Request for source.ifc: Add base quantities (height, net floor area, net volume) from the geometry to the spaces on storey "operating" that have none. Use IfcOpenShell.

First a look at what the model holds.

```python
import ifcopenshell
import ifcopenshell.util.element
import ifcopenshell.util.unit

model = ifcopenshell.open("source.ifc")
print(model.schema)
for unit_type in ("LENGTHUNIT", "AREAUNIT", "VOLUMEUNIT"):
    print(unit_type, ifcopenshell.util.unit.calculate_unit_scale(model, unit_type))
storey = next(s for s in model.by_type("IfcBuildingStorey") if s.Name == "operating")
spaces = [e for e in ifcopenshell.util.element.get_decomposition(storey) if e.is_a("IfcSpace")]
for e in sorted(spaces, key=lambda e: e.id()):
    print(e.id(), e.is_a(), e.Name, list(ifcopenshell.util.element.get_psets(e, qtos_only=True)), sep=" | ")
```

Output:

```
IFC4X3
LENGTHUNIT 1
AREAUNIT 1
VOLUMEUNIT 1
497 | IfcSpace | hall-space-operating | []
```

```python
import ifcopenshell
import ifcopenshell.api.pset
import ifcopenshell.geom
import ifcopenshell.util.element
import ifcopenshell.util.shape
import ifcopenshell.util.unit

model = ifcopenshell.open("source.ifc")
unit_scale = ifcopenshell.util.unit.calculate_unit_scale(model)
area_scale = ifcopenshell.util.unit.calculate_unit_scale(model, "AREAUNIT")
volume_scale = ifcopenshell.util.unit.calculate_unit_scale(model, "VOLUMEUNIT")
settings = ifcopenshell.geom.settings()

storey = next(s for s in model.by_type("IfcBuildingStorey") if s.Name == "operating")
spaces = [e for e in ifcopenshell.util.element.get_decomposition(storey) if e.is_a("IfcSpace")]

for e in sorted(spaces, key=lambda e: e.id()):
    if ifcopenshell.util.element.get_psets(e, qtos_only=True, should_inherit=False):
        continue
    # Geometry comes back in metres, in the element's own axes.
    shape = ifcopenshell.geom.create_shape(settings, e)
    values = {
        "Height": ifcopenshell.util.shape.get_z(shape.geometry) / unit_scale,
        "NetFloorArea": ifcopenshell.util.shape.get_footprint_area(shape.geometry) / area_scale,
        "NetVolume": ifcopenshell.util.shape.get_volume(shape.geometry) / volume_scale,
    }
    qto = ifcopenshell.api.pset.add_qto(model, product=e, name="Qto_SpaceBaseQuantities")
    ifcopenshell.api.pset.edit_qto(model, qto=qto, properties=values)
    print(e.id(), {k: round(v, 3) for k, v in values.items()})

model.write("source_rev.ifc")
```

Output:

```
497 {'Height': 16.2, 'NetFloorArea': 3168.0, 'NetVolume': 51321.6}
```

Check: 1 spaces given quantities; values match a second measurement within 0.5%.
